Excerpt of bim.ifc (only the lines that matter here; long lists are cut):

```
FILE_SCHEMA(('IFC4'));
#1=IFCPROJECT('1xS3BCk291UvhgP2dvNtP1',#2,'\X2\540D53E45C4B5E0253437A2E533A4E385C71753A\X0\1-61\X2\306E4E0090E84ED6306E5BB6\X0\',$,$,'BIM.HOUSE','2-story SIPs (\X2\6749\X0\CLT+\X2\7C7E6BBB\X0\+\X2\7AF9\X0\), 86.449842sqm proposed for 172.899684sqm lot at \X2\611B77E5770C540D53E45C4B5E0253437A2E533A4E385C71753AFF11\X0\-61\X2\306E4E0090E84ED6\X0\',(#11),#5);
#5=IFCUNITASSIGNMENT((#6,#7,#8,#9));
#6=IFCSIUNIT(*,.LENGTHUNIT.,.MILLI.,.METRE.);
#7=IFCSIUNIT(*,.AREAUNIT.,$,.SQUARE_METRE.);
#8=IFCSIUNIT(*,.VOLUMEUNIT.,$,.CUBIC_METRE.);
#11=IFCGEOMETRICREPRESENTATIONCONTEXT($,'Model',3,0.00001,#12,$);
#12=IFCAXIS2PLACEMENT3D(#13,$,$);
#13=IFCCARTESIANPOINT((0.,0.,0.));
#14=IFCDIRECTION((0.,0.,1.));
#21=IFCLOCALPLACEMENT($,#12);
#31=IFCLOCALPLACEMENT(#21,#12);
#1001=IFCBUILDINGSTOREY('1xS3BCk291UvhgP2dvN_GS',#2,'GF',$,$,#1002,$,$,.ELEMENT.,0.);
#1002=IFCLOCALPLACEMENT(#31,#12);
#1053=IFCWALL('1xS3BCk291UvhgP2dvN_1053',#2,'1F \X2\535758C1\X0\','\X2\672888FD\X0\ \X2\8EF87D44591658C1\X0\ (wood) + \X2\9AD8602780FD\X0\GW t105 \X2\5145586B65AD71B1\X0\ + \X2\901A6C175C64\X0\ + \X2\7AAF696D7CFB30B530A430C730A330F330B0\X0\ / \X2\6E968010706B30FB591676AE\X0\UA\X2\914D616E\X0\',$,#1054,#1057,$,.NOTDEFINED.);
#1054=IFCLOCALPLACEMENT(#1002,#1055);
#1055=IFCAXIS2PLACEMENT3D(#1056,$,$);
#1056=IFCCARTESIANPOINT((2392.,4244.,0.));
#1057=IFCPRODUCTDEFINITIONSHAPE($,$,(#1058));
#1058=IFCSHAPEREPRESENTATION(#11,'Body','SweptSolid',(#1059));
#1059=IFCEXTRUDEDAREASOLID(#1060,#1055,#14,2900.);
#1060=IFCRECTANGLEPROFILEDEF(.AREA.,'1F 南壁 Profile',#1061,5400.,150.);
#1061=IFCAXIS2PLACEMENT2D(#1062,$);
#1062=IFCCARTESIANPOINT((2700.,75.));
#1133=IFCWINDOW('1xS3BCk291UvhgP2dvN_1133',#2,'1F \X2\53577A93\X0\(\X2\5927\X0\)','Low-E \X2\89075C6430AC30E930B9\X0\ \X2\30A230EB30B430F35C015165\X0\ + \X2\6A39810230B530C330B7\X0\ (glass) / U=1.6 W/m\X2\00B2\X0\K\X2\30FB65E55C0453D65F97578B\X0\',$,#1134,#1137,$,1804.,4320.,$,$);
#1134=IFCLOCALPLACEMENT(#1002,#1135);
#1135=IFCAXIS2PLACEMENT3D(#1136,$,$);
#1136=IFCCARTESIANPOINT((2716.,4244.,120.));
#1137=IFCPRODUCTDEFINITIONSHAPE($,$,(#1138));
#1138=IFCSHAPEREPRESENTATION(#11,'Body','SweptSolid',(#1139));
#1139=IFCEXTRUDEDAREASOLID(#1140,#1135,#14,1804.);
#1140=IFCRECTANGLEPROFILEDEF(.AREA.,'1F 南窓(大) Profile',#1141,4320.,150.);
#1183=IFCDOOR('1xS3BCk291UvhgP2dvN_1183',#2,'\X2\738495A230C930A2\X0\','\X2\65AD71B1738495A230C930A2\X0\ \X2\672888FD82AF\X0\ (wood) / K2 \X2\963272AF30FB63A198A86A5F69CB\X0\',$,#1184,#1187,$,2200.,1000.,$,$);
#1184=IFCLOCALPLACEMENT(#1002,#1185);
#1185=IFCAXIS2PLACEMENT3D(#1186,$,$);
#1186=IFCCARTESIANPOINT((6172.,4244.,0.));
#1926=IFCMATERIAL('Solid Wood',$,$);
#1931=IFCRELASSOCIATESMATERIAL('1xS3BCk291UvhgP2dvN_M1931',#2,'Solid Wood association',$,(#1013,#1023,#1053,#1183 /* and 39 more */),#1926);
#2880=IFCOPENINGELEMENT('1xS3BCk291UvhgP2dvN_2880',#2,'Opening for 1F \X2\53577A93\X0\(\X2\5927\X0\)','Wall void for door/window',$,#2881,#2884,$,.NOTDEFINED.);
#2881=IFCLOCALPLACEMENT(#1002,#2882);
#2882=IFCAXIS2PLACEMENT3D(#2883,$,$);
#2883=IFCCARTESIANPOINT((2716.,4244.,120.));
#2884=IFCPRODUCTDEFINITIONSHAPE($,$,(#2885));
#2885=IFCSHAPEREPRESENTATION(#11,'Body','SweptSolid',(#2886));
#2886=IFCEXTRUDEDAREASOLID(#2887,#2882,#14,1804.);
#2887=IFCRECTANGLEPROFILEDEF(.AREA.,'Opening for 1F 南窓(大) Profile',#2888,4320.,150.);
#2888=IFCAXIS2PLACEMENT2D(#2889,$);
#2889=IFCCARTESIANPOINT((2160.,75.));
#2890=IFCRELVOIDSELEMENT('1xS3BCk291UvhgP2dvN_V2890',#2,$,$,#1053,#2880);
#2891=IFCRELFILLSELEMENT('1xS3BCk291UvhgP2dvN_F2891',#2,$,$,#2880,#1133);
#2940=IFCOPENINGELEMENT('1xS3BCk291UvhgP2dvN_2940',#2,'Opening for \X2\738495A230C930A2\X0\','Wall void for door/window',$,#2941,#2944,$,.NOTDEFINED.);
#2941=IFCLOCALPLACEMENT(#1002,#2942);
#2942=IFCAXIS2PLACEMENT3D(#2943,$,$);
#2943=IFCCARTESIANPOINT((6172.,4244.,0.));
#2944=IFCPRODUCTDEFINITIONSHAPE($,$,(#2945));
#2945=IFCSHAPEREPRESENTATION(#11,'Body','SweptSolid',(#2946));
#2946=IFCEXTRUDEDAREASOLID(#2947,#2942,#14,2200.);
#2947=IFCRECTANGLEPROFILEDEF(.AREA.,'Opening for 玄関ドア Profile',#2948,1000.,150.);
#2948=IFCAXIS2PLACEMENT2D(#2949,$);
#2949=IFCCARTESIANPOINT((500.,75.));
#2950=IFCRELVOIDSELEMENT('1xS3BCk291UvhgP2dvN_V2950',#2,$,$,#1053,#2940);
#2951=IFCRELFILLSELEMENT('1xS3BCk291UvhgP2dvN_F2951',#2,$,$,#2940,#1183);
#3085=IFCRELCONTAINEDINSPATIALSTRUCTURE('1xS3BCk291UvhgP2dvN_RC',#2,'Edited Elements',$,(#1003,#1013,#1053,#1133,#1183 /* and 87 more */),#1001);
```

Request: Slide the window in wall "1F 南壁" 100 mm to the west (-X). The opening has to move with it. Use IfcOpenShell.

```python
import ifcopenshell
import ifcopenshell.api.geometry
import ifcopenshell.util.placement
import ifcopenshell.util.unit

model = ifcopenshell.open("bim.ifc")
unit_scale = ifcopenshell.util.unit.calculate_unit_scale(model)

window = model.by_guid("1xS3BCk291UvhgP2dvN_1133")
opening = window.FillsVoids[0].RelatingOpeningElement
wall = opening.VoidsElements[0].RelatingBuildingElement

wall_matrix = ifcopenshell.util.placement.get_local_placement(wall.ObjectPlacement)
shift = wall_matrix[:3, 0] * -0.1 / unit_scale
before = ifcopenshell.util.placement.get_local_placement(window.ObjectPlacement)[:3, 3].copy()

# The window is not placed relative to its opening, so move both.
for product in (opening, window):
    matrix = ifcopenshell.util.placement.get_local_placement(product.ObjectPlacement)
    matrix[:3, 3] += shift
    ifcopenshell.api.geometry.edit_object_placement(model, product=product, matrix=matrix, is_si=False)

after = ifcopenshell.util.placement.get_local_placement(window.ObjectPlacement)[:3, 3]
print("window moved by", (after - before).round(3) + 0.0)

model.write("bim_v2.ifc")
```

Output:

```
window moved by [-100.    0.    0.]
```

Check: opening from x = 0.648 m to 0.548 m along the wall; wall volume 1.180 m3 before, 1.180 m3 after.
